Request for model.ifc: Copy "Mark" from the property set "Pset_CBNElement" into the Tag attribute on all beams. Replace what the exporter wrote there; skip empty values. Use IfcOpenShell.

First a look at what the model holds.

```python
import ifcopenshell
import ifcopenshell.util.element

model = ifcopenshell.open("model.ifc")
print(model.schema)
beams = model.by_type("IfcBeam")
print(len(beams), "beams")
for e in beams[:8]:
    source = ifcopenshell.util.element.get_pset(e, "Pset_CBNElement", "Mark")
    target = e.Tag
    print(e.id(), repr(source), repr(target), sep=" | ")
```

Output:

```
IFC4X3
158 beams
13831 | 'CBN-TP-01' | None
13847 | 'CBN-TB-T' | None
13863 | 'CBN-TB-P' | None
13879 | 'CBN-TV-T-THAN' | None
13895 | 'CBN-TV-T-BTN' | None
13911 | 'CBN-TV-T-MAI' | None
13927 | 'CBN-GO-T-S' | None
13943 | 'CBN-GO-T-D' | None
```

```python
import ifcopenshell
import ifcopenshell.util.element

model = ifcopenshell.open("model.ifc")

count = 0
for e in model.by_type("IfcBeam"):
    value = ifcopenshell.util.element.get_pset(e, "Pset_CBNElement", "Mark")
    current = e.Tag
    if not value or not value.strip() or current == value:
        continue
    e.Tag = value
    count += 1

print(count, "beams updated")

model.write("model-out.ifc")
```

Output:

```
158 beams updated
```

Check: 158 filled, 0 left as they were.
